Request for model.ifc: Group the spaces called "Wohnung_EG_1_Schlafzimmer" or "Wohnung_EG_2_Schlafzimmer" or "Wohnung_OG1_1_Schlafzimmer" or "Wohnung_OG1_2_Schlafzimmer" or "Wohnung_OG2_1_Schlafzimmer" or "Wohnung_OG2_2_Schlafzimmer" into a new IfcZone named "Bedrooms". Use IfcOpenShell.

First a look at what the model holds.

```python
import ifcopenshell

model = ifcopenshell.open("model.ifc")
print(model.schema)
seen = {}
for space in model.by_type("IfcSpace"):
    seen[space.LongName] = seen.get(space.LongName, 0) + 1
for name, count in sorted(seen.items(), key=str):
    print(count, "x", name)
print("zones:", [z.Name for z in model.by_type("IfcZone")][:20])
```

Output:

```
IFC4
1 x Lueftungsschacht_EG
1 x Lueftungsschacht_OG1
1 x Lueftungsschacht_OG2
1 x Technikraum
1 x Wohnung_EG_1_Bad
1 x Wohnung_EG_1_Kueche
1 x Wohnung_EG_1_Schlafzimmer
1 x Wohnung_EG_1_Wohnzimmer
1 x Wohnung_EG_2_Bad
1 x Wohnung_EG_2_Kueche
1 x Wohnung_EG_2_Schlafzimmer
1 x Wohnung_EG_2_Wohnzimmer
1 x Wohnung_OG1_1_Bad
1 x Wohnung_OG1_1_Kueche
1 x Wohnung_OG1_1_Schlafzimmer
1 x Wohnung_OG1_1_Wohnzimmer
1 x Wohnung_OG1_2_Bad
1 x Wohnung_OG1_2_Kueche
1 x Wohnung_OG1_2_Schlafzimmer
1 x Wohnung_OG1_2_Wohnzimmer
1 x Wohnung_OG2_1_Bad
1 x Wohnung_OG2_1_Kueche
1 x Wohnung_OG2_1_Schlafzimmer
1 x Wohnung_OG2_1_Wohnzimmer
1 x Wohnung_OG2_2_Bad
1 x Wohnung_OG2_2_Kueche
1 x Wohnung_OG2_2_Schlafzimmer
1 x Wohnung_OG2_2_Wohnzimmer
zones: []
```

```python
import ifcopenshell
import ifcopenshell.api.group
import ifcopenshell.api.root

model = ifcopenshell.open("model.ifc")

names = {"Wohnung_EG_1_Schlafzimmer", "Wohnung_EG_2_Schlafzimmer", "Wohnung_OG1_1_Schlafzimmer", "Wohnung_OG1_2_Schlafzimmer", "Wohnung_OG2_1_Schlafzimmer", "Wohnung_OG2_2_Schlafzimmer"}
spaces = [s for s in model.by_type("IfcSpace") if s.LongName in names]

zone = ifcopenshell.api.root.create_entity(model, ifc_class="IfcZone", name="Bedrooms")
ifcopenshell.api.group.assign_group(model, products=spaces, group=zone)
print(len(spaces), "spaces in", zone.Name)

model.write("model_edited.ifc")
```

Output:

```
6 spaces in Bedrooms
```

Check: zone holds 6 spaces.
